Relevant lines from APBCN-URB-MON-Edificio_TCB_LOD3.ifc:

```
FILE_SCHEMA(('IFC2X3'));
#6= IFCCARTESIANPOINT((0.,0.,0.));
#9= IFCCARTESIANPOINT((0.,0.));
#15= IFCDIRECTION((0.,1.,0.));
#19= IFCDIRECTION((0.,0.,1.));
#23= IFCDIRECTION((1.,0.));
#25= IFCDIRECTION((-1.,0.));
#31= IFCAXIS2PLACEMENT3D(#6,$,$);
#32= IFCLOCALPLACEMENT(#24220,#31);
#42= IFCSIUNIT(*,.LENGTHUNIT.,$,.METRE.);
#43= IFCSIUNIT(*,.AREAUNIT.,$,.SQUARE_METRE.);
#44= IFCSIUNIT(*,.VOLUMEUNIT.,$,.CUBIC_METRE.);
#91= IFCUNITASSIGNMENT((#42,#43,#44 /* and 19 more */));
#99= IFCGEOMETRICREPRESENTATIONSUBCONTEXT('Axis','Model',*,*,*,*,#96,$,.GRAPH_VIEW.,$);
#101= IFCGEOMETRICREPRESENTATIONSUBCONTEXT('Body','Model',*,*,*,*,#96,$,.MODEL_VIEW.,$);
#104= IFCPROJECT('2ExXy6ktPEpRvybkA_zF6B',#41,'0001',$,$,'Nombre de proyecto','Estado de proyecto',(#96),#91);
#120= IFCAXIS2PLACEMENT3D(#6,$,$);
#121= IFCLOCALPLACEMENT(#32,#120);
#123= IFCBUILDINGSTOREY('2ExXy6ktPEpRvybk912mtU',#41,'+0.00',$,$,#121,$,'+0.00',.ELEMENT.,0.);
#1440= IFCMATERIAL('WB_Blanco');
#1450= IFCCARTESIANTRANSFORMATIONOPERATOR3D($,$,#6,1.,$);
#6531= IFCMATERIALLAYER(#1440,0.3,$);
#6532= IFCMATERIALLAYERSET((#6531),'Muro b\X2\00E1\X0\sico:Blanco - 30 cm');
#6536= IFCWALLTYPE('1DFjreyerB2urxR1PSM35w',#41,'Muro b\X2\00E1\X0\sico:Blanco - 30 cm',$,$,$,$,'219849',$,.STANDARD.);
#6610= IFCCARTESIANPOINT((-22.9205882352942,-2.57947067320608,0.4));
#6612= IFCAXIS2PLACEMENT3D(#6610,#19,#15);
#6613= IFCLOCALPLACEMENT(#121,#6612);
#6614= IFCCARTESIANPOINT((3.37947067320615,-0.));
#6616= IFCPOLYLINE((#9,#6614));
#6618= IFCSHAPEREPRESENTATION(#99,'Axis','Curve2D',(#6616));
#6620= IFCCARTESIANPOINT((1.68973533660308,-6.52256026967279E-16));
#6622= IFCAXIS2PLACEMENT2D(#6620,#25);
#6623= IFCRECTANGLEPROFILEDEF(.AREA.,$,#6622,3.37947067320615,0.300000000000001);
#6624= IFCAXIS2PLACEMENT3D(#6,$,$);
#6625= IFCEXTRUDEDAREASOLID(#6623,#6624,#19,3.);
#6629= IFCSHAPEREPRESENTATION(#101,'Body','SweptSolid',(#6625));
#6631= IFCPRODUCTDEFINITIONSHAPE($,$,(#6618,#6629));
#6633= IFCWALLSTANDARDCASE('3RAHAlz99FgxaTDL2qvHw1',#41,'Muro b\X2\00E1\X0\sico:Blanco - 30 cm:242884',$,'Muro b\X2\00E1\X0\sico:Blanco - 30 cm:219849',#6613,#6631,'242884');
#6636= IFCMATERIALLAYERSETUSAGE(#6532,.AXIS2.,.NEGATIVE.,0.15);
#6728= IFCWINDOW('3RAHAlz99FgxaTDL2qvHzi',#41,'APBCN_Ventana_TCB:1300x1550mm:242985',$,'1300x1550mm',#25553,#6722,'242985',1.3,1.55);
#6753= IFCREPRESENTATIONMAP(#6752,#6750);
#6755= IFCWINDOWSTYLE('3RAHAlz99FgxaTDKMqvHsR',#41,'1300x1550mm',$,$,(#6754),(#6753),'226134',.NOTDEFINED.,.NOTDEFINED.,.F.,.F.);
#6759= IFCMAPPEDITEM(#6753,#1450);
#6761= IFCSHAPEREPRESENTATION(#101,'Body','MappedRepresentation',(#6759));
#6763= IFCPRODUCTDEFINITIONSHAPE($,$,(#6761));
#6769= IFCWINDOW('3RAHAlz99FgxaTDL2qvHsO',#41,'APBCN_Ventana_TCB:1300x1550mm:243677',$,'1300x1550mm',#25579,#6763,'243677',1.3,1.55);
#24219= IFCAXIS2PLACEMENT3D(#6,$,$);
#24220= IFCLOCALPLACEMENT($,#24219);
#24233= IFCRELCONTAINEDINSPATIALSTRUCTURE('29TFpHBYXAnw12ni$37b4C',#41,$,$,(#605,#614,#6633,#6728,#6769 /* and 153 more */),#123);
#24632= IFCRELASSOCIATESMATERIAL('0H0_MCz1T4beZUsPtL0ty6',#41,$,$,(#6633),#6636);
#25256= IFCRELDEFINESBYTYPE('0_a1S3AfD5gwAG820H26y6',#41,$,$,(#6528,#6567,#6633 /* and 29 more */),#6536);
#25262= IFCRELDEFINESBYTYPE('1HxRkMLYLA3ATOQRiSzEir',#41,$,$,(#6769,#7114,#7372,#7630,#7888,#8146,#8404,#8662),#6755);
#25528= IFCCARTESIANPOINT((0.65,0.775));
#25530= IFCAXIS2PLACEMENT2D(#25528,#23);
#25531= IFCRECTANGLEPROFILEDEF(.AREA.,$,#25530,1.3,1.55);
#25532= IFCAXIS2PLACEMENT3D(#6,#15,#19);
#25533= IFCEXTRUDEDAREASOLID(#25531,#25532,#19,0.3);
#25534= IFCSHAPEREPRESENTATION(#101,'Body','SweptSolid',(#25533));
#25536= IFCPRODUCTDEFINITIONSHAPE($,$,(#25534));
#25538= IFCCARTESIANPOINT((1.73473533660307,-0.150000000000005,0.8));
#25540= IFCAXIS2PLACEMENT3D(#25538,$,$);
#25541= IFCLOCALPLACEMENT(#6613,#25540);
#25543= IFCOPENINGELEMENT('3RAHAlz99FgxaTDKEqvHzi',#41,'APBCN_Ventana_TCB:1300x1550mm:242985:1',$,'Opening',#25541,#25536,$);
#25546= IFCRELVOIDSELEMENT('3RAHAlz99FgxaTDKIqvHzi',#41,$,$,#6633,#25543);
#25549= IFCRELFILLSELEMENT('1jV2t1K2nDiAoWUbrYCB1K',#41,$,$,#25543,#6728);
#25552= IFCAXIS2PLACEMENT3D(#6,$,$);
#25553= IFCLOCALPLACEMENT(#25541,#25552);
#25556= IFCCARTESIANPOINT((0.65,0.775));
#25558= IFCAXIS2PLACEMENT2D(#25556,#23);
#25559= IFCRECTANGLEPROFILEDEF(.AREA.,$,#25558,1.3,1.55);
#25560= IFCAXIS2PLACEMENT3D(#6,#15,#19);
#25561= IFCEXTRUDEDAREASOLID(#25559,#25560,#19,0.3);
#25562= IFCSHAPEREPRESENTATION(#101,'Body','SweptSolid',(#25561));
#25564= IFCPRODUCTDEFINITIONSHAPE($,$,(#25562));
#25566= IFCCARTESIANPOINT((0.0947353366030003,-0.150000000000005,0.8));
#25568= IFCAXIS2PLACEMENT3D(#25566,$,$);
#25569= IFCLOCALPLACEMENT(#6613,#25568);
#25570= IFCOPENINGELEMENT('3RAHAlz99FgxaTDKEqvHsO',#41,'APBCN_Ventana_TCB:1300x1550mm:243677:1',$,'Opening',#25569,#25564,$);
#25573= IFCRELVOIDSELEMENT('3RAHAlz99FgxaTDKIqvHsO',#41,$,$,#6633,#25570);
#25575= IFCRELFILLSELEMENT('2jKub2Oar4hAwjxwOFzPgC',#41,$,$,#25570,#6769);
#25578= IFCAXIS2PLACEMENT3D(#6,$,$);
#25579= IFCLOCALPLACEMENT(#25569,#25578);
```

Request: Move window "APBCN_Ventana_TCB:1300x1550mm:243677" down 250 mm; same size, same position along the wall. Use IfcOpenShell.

```python
import numpy as np
import ifcopenshell
import ifcopenshell.api.geometry
import ifcopenshell.util.placement
import ifcopenshell.util.unit

model = ifcopenshell.open("APBCN-URB-MON-Edificio_TCB_LOD3.ifc")
unit_scale = ifcopenshell.util.unit.calculate_unit_scale(model)

window = model.by_id(6769)
opening = window.FillsVoids[0].RelatingOpeningElement
dz = -0.25

shift = np.array([0.0, 0.0, dz])
# The window is placed relative to its opening, so it follows when the opening moves.
matrix = ifcopenshell.util.placement.get_local_placement(opening.ObjectPlacement)
matrix[:3, 3] += shift
ifcopenshell.api.geometry.edit_object_placement(
    model, product=opening, matrix=matrix, is_si=False, should_transform_children=True
)

print(f"moved by {dz * unit_scale:+.3f} m")

model.write("APBCN-URB-MON-Edificio_TCB_LOD3-out.ifc")
```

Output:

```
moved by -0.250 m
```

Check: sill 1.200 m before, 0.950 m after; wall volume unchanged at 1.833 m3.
